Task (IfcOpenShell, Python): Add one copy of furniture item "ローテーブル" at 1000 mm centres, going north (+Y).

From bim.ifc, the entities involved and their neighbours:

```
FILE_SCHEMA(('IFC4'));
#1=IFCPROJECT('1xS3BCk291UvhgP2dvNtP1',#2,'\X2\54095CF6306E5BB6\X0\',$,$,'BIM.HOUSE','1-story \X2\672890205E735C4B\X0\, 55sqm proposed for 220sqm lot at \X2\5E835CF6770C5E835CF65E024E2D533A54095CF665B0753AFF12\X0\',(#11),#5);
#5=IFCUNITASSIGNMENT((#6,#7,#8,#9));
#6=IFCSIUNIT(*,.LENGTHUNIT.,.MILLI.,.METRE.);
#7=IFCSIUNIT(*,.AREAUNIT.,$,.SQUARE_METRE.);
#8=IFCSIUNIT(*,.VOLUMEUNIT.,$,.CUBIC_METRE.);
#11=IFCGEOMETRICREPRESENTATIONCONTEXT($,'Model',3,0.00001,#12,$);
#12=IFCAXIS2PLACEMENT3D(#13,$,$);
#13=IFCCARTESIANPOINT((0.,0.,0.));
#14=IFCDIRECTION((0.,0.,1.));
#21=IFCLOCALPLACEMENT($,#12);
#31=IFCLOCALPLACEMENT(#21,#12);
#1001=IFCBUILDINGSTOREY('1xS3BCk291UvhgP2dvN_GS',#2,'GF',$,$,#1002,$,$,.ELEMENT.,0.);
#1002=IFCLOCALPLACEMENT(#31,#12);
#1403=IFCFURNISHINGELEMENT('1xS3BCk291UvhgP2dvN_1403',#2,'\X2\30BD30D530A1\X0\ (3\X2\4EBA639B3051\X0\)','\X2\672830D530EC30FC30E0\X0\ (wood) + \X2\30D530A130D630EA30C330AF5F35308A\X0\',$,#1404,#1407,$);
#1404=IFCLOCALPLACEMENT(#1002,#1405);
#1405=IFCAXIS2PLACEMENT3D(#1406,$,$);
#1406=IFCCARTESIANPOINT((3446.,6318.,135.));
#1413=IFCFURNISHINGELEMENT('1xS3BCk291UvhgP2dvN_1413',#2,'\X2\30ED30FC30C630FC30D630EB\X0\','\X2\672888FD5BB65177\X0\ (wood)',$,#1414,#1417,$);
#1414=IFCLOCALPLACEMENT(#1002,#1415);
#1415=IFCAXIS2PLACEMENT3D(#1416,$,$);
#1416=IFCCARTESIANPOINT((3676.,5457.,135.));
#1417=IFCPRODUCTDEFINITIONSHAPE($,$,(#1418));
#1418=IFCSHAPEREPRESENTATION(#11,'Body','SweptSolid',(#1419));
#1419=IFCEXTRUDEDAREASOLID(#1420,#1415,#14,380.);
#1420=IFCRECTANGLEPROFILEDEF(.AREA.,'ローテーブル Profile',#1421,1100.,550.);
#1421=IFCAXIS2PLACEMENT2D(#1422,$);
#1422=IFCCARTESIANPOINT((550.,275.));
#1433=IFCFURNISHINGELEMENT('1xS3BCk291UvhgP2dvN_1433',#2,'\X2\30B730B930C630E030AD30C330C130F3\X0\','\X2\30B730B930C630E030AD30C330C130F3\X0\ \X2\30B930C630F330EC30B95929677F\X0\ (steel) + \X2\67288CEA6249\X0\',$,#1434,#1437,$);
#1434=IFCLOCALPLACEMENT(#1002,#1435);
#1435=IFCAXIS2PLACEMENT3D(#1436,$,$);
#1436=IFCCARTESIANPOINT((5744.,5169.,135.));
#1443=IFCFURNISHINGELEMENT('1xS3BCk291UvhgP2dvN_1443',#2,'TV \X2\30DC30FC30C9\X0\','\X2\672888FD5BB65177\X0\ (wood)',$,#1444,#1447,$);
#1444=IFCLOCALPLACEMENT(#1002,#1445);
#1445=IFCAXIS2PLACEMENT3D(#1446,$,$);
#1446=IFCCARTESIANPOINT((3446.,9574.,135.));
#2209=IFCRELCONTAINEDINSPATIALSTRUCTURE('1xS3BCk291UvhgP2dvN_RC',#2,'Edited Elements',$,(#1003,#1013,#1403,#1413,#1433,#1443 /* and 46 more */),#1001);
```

```python
import numpy as np
import ifcopenshell
import ifcopenshell.api.geometry
import ifcopenshell.api.root
import ifcopenshell.util.element
import ifcopenshell.util.placement
import ifcopenshell.util.unit

model = ifcopenshell.open("bim.ifc")
unit_scale = ifcopenshell.util.unit.calculate_unit_scale(model)


def reuse_history(source, copy):
    """copy_class also copies each property set's owner history, people and application; keep the originals."""
    for rel in copy.IsDefinedBy:
        if rel.is_a("IfcRelDefinesByProperties") and (history := rel.RelatingPropertyDefinition.OwnerHistory):
            rel.RelatingPropertyDefinition.OwnerHistory = source.OwnerHistory
            ifcopenshell.util.element.remove_deep2(model, history)


source = model.by_guid("1xS3BCk291UvhgP2dvN_1413")
base = ifcopenshell.util.placement.get_local_placement(source.ObjectPlacement)
step = np.array([0.0, 1.0, 0.0]) * 1 / unit_scale

for i in range(1, 2):
    copy = ifcopenshell.api.root.copy_class(model, product=source)
    copy.Representation = ifcopenshell.util.element.copy_deep(
        model, source.Representation, exclude=["IfcGeometricRepresentationContext", "IfcRepresentationMap"]
    )
    reuse_history(source, copy)
    matrix = base.copy()
    matrix[:3, 3] += i * step
    print("added at", matrix[:3, 3].round(3) + 0.0)
    ifcopenshell.api.geometry.edit_object_placement(model, product=copy, matrix=matrix, is_si=False)

model.write("bim-out.ifc")
```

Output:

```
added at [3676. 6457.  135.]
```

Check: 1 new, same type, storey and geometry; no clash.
